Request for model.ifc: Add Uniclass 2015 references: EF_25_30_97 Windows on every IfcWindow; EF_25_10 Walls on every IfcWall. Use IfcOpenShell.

First a look at what the model holds.

```python
import ifcopenshell

model = ifcopenshell.open("model.ifc")
print(model.schema)
print("classifications:", [c.Name for c in model.by_type("IfcClassification")])
for ifc_class in ("IfcDoor", "IfcRoof", "IfcStair", "IfcWall", "IfcWindow"):
    print(ifc_class, len(model.by_type(ifc_class)))
```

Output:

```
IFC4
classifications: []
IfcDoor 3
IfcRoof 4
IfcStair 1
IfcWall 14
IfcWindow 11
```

```python
import ifcopenshell
import ifcopenshell.api.classification

model = ifcopenshell.open("model.ifc")

system = ifcopenshell.api.classification.add_classification(model, classification="Uniclass 2015")

codes = {
    "IfcWindow": ("EF_25_30_97", "Windows"),
    "IfcWall": ("EF_25_10", "Walls"),
}
for ifc_class, (code, name) in codes.items():
    products = model.by_type(ifc_class)
    ifcopenshell.api.classification.add_reference(
        model, products=products, classification=system, identification=code, name=name
    )
    print(code, len(products))

model.write("model_rev.ifc")
```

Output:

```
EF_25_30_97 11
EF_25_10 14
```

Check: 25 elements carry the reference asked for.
